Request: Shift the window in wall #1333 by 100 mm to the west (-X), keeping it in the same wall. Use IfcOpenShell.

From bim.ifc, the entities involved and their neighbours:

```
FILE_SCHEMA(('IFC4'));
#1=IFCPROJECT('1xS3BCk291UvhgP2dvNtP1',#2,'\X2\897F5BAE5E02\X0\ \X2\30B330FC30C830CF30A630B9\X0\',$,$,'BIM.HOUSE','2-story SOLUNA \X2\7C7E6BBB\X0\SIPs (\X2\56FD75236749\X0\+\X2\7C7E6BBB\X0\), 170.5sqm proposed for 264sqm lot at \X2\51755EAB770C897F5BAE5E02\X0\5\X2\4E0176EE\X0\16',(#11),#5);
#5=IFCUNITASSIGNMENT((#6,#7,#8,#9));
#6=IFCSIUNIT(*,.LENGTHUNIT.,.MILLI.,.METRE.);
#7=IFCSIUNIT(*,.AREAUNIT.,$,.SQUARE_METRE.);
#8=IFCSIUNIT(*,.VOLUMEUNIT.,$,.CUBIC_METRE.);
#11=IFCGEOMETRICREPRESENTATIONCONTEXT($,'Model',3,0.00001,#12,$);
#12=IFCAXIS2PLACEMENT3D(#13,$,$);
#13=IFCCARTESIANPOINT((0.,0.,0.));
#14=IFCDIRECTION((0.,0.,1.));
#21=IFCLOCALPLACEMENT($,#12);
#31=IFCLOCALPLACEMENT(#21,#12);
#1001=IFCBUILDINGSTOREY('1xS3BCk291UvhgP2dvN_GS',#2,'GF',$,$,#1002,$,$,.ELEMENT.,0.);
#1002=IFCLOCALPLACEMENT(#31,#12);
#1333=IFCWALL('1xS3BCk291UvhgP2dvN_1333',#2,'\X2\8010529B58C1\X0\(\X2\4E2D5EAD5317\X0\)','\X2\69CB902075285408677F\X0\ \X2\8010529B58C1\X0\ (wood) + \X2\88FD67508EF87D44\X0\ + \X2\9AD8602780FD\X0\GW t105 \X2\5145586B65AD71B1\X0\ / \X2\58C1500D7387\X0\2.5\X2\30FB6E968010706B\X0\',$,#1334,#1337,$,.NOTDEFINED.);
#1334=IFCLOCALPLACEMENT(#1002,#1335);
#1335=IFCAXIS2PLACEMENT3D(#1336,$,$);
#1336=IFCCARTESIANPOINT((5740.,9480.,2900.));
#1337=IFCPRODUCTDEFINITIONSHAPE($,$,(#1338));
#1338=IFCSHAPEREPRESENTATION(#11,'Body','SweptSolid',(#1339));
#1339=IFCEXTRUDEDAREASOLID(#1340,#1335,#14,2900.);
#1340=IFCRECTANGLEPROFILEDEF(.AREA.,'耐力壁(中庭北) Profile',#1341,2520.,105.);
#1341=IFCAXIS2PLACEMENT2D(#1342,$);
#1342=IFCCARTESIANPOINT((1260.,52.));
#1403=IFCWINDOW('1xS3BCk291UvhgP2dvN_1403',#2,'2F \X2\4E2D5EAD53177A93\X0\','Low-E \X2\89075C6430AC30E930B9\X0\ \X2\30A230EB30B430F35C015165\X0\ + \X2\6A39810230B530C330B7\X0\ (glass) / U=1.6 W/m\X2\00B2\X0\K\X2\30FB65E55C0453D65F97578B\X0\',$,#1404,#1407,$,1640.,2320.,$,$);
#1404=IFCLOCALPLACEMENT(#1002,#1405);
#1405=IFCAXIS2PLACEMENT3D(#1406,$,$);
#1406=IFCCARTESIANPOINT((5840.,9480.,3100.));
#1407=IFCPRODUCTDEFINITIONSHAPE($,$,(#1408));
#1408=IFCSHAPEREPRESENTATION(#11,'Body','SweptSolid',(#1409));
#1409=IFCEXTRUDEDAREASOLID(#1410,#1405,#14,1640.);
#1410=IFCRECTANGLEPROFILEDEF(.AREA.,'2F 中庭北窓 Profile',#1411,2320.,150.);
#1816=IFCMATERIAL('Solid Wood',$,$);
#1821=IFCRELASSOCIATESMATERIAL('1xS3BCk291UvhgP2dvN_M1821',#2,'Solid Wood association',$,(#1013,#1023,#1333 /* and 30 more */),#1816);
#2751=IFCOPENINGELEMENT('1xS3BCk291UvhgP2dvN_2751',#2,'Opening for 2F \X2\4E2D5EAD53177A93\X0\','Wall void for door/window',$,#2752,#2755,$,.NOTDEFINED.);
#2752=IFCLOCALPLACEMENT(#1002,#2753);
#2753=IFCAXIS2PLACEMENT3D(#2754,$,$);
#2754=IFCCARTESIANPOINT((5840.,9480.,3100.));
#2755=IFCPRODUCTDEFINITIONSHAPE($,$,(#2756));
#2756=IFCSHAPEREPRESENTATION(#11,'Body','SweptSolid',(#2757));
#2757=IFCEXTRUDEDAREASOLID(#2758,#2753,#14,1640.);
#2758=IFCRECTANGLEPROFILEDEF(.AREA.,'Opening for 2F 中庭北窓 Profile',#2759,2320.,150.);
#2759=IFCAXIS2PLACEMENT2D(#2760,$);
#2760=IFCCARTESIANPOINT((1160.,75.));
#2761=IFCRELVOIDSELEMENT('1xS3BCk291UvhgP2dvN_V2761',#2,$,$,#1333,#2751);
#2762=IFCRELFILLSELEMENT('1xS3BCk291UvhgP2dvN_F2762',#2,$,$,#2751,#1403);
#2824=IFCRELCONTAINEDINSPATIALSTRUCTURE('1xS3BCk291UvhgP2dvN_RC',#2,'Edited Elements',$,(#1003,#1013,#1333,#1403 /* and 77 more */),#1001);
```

```python
import ifcopenshell
import ifcopenshell.api.geometry
import ifcopenshell.util.placement

model = ifcopenshell.open("bim.ifc")

window = model.by_guid("1xS3BCk291UvhgP2dvN_1403")
opening = window.FillsVoids[0].RelatingOpeningElement
wall = opening.VoidsElements[0].RelatingBuildingElement

wall_matrix = ifcopenshell.util.placement.get_local_placement(wall.ObjectPlacement)
shift = wall_matrix[:3, 0] * -100.0
before = ifcopenshell.util.placement.get_local_placement(window.ObjectPlacement)[:3, 3].copy()

# The window is not placed relative to its opening, so move both.
for product in (opening, window):
    matrix = ifcopenshell.util.placement.get_local_placement(product.ObjectPlacement)
    matrix[:3, 3] += shift
    ifcopenshell.api.geometry.edit_object_placement(model, product=product, matrix=matrix, is_si=False)

after = ifcopenshell.util.placement.get_local_placement(window.ObjectPlacement)[:3, 3]
print("window moved by", (after - before).round(3) + 0.0)

model.write("bim-out.ifc")
```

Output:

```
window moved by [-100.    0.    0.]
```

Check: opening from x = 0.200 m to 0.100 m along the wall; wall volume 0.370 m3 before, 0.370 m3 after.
